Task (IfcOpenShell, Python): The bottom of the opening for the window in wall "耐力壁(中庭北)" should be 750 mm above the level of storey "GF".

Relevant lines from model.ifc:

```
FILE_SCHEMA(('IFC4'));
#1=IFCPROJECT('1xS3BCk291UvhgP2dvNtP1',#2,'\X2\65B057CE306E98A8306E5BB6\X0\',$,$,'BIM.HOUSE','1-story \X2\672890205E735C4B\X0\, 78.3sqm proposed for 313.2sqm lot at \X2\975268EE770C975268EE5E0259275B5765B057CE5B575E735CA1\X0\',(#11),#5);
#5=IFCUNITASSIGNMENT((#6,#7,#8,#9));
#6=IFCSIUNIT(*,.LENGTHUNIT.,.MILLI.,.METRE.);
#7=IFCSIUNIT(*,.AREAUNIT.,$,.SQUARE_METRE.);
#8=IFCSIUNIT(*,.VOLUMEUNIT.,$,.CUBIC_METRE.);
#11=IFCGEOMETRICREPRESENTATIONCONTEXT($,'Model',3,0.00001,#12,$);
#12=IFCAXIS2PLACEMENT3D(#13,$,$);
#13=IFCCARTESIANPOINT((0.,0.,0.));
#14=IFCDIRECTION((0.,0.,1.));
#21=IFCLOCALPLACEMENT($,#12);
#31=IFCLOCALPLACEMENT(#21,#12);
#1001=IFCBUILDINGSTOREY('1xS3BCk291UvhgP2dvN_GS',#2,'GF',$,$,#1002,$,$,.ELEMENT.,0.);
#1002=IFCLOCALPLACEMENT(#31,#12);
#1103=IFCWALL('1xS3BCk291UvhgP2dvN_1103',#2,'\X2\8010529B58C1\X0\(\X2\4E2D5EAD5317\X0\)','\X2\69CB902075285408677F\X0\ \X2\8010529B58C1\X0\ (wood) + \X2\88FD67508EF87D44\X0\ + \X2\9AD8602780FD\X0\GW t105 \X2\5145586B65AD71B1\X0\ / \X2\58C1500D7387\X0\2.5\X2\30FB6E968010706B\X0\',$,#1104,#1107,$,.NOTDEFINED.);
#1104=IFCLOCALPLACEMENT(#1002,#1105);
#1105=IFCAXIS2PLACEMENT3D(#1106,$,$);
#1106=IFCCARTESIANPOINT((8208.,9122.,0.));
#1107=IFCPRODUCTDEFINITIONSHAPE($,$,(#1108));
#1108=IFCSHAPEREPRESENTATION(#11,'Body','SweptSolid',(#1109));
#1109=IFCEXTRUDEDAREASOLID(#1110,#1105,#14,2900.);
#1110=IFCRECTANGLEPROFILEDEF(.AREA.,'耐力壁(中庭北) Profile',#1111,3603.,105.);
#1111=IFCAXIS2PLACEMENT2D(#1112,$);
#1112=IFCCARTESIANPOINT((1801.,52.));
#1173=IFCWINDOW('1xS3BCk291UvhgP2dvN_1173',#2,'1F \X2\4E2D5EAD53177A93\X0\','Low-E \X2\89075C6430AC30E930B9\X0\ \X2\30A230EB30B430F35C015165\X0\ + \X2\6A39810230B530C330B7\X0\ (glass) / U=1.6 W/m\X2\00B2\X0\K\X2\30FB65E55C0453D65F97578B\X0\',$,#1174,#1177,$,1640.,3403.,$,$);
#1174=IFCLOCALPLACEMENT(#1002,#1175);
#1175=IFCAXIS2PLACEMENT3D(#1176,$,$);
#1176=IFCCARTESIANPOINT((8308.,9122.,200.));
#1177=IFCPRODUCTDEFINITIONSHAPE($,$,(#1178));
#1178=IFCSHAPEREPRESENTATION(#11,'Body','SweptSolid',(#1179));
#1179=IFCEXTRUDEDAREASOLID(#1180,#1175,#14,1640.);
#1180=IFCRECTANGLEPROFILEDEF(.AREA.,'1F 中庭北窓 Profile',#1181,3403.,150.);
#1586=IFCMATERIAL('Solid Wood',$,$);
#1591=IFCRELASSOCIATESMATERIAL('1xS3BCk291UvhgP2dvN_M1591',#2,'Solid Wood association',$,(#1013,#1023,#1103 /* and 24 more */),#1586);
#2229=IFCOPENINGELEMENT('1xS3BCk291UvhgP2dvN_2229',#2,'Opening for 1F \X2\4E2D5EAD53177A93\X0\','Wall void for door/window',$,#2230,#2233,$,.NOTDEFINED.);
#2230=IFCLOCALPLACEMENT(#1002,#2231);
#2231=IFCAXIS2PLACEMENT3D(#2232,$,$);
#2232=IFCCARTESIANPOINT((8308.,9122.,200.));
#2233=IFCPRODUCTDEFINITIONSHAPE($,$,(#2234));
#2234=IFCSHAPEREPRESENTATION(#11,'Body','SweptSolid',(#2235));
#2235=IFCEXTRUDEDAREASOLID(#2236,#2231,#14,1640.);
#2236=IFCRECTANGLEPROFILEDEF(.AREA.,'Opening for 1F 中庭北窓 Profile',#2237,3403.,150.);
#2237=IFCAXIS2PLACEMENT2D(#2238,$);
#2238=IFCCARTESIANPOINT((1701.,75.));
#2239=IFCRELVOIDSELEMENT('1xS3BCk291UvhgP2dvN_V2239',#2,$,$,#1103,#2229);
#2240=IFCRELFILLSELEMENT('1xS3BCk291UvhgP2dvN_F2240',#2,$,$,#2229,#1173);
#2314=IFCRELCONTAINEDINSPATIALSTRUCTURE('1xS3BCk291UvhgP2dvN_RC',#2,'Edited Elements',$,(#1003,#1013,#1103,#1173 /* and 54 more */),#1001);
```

```python
import numpy as np
import ifcopenshell
import ifcopenshell.api.geometry
import ifcopenshell.geom
import ifcopenshell.util.element
import ifcopenshell.util.placement
import ifcopenshell.util.shape
import ifcopenshell.util.unit

model = ifcopenshell.open("model.ifc")
unit_scale = ifcopenshell.util.unit.calculate_unit_scale(model)

window = model.by_guid("1xS3BCk291UvhgP2dvN_1173")
opening = window.FillsVoids[0].RelatingOpeningElement
storey = ifcopenshell.util.element.get_container(window, ifc_class="IfcBuildingStorey")
level = ifcopenshell.util.placement.get_local_placement(storey.ObjectPlacement)[2, 3]

# The opening's origin need not be at the sill, so measure its lowest point.
shape = ifcopenshell.geom.create_shape(ifcopenshell.geom.settings(), opening)
bottom = ifcopenshell.util.shape.get_shape_bottom_elevation(shape, shape.geometry) / unit_scale
dz = level + 0.75 / unit_scale - bottom

shift = np.array([0.0, 0.0, dz])
# The window is not placed relative to its opening, so move both.
for product in (opening, window):
    matrix = ifcopenshell.util.placement.get_local_placement(product.ObjectPlacement)
    matrix[:3, 3] += shift
    ifcopenshell.api.geometry.edit_object_placement(model, product=product, matrix=matrix, is_si=False)

print(f"moved by {dz * unit_scale:+.3f} m")

model.write("model_rev.ifc")
```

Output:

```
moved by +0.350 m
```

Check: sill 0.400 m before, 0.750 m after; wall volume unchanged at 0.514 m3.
